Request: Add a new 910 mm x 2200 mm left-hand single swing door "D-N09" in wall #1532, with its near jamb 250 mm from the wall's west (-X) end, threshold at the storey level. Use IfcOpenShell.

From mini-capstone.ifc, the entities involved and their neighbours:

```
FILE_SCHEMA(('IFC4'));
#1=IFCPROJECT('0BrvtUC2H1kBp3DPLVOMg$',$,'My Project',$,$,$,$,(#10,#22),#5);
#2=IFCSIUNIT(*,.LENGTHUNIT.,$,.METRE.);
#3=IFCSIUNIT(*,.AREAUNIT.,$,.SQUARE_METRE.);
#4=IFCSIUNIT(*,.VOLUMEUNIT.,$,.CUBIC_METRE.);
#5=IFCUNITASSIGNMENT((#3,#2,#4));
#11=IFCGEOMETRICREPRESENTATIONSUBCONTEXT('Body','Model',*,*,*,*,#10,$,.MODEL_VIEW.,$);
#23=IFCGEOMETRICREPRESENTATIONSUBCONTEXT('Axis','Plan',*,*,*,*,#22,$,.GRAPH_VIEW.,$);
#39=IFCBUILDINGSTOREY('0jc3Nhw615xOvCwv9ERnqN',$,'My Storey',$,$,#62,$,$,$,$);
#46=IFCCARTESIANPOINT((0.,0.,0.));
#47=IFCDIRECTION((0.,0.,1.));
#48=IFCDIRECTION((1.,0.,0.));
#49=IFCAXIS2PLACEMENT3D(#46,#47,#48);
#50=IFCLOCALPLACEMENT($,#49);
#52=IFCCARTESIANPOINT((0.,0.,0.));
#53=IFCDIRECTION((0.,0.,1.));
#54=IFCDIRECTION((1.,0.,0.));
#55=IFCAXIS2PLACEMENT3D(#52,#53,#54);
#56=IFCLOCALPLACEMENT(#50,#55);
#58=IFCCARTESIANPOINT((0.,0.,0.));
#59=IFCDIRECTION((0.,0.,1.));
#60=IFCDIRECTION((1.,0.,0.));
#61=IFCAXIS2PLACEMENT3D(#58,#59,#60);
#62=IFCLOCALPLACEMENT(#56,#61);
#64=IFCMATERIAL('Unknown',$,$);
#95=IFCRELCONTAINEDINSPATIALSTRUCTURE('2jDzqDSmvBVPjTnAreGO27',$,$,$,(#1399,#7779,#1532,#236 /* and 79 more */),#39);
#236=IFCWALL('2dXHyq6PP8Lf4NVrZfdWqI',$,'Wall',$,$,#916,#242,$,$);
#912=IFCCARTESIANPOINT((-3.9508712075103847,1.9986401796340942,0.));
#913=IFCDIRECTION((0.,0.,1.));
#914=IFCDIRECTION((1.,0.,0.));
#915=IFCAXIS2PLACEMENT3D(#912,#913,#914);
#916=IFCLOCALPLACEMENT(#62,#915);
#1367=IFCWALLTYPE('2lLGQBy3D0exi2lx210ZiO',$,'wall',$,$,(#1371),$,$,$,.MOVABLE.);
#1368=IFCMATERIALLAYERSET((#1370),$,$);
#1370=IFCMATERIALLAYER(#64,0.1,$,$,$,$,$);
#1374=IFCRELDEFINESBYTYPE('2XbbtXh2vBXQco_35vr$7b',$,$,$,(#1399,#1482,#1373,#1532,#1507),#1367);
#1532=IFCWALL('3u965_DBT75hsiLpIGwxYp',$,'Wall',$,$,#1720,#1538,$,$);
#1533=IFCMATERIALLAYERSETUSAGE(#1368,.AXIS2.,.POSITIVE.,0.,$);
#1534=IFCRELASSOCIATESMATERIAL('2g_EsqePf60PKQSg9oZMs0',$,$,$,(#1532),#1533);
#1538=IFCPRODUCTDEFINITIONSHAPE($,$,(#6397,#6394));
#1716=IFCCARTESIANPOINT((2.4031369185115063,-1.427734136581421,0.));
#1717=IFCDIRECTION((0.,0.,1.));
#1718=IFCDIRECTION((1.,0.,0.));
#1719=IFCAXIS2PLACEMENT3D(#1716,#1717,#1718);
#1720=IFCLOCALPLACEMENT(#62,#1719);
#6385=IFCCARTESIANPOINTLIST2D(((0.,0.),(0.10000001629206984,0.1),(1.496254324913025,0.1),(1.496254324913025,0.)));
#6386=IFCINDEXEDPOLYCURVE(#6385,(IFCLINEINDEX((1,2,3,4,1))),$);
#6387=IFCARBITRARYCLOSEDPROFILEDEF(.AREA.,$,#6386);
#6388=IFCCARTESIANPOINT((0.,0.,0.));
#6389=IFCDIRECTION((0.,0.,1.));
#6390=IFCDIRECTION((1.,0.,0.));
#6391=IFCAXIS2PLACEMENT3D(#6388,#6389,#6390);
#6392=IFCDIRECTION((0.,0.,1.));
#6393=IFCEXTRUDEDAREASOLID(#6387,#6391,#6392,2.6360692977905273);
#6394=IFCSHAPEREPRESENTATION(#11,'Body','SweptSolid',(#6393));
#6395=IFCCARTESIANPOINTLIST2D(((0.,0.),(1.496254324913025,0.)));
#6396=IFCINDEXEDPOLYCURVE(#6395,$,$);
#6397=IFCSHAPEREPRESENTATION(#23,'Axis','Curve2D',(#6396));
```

```python
import numpy as np
import ifcopenshell
import ifcopenshell.api.feature
import ifcopenshell.api.geometry
import ifcopenshell.api.root
import ifcopenshell.api.spatial
import ifcopenshell.geom
import ifcopenshell.util.element
import ifcopenshell.util.placement
import ifcopenshell.util.representation
import ifcopenshell.util.shape
import ifcopenshell.util.unit

model = ifcopenshell.open("mini-capstone.ifc")
unit_scale = ifcopenshell.util.unit.calculate_unit_scale(model)
settings = ifcopenshell.geom.settings()


def volume(element):
    """Net volume in cubic metres, openings subtracted."""
    shape = ifcopenshell.geom.create_shape(settings, element)
    return ifcopenshell.util.shape.get_volume(shape.geometry)


wall = model.by_guid("3u965_DBT75hsiLpIGwxYp")
storey = ifcopenshell.util.element.get_container(wall, ifc_class="IfcBuildingStorey")
context = ifcopenshell.util.representation.get_context(model, "Model", "Body", "MODEL_VIEW")
before = volume(wall)

width, height, from_end, sill = 0.91, 2.2, 0.25, 0.0  # metres

# The wall runs along its own X axis, and the end named is its -X end.
wall_shape = ifcopenshell.geom.create_shape(settings, wall)
x, y, z = ifcopenshell.util.shape.get_vertices(wall_shape.geometry).T
start = x.min() + from_end
face, thickness = float(y.min()), float(y.max() - y.min())
wall_matrix = ifcopenshell.util.placement.get_local_placement(wall.ObjectPlacement)
level = ifcopenshell.util.placement.get_local_placement(storey.ObjectPlacement)[2, 3]


def in_wall(x, y):
    """Placement at x, y metres in the wall's axes, at sill height."""
    matrix = wall_matrix.copy()
    matrix[:, 3] = wall_matrix @ np.array([x / unit_scale, y / unit_scale, 0.0, 1.0])
    matrix[2, 3] = level + sill / unit_scale
    return matrix


# Opening: a box that overshoots both wall faces by 50 mm.
opening = ifcopenshell.api.root.create_entity(model, ifc_class="IfcOpeningElement", predefined_type="OPENING")
box = ifcopenshell.api.geometry.add_wall_representation(
    model, context=context, length=width, height=height, thickness=thickness + 0.1
)
ifcopenshell.api.geometry.assign_representation(model, product=opening, representation=box)
ifcopenshell.api.geometry.edit_object_placement(model, product=opening, matrix=in_wall(start, face - 0.05), is_si=False)
ifcopenshell.api.feature.add_feature(model, feature=opening, element=wall)

door = ifcopenshell.api.root.create_entity(model, ifc_class="IfcDoor", name="D-N09", predefined_type="DOOR")
door.OverallWidth, door.OverallHeight = width / unit_scale, height / unit_scale
door.OperationType = "SINGLE_SWING_LEFT"
body = ifcopenshell.api.geometry.add_door_representation(
    model,
    context=context,
    overall_width=door.OverallWidth,
    overall_height=door.OverallHeight,
    operation_type="SINGLE_SWING_LEFT",
    lining_properties={"LiningDepth": thickness / unit_scale, "ThresholdDepth": thickness / unit_scale},
)
ifcopenshell.api.geometry.assign_representation(model, product=door, representation=body)
ifcopenshell.api.spatial.assign_container(model, products=[door], relating_structure=storey)
ifcopenshell.api.feature.add_filling(model, opening=opening, element=door)

# The lining spans the wall, so the door starts at the wall face.
ifcopenshell.api.geometry.edit_object_placement(model, product=door, matrix=in_wall(start, face), is_si=False)

after = volume(wall)

print(f"wall volume {before:.3f} -> {after:.3f} m3")

model.write("mini-capstone_rev.ifc")
```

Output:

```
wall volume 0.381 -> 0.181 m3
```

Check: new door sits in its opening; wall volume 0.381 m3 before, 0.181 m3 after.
